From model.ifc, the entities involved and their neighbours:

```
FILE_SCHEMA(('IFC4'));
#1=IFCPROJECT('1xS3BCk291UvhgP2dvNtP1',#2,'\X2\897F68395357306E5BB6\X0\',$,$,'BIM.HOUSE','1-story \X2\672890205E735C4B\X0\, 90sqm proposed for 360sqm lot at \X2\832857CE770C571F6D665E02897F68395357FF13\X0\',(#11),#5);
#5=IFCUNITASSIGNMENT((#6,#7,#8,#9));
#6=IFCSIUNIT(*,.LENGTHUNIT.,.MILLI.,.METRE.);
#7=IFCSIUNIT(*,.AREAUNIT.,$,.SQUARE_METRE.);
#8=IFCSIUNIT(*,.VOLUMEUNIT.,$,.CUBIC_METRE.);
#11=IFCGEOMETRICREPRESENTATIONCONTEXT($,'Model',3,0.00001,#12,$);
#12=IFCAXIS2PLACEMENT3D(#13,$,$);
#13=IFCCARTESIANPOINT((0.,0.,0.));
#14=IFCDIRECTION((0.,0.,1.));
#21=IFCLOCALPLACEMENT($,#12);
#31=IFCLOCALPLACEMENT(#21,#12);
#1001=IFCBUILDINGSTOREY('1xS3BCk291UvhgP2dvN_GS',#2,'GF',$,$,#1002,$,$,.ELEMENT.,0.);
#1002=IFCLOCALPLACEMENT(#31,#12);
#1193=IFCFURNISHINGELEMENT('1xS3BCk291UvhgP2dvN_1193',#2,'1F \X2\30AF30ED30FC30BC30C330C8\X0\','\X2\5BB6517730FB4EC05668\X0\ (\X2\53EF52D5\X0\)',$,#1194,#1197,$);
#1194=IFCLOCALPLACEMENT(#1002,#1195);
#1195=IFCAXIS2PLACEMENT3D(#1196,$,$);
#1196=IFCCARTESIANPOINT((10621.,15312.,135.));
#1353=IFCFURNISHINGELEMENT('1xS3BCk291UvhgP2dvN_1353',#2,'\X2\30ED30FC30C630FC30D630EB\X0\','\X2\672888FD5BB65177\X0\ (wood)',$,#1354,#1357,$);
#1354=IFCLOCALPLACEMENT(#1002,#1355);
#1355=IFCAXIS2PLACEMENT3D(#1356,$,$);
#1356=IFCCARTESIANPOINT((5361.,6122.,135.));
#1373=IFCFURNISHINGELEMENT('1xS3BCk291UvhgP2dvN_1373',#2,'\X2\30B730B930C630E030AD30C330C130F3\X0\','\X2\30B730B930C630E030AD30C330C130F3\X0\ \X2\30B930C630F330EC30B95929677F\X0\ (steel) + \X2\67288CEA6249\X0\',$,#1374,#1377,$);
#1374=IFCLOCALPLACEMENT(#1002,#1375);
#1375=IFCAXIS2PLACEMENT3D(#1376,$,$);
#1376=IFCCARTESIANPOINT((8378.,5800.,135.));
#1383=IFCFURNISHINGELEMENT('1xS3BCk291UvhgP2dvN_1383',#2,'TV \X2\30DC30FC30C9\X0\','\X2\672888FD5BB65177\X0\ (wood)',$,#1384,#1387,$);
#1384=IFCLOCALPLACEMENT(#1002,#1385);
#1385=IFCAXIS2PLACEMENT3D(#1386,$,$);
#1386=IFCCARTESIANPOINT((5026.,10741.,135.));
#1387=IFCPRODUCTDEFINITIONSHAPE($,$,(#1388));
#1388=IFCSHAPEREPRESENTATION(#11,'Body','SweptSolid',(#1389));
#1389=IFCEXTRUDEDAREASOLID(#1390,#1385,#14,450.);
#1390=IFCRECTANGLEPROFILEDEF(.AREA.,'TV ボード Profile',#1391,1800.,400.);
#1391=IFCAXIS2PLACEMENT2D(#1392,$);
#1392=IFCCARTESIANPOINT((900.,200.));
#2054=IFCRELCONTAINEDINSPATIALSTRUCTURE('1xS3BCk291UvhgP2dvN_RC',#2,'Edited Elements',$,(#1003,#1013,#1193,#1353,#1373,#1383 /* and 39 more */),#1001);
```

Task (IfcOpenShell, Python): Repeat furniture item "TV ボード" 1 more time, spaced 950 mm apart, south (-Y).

```python
import numpy as np
import ifcopenshell
import ifcopenshell.api.geometry
import ifcopenshell.api.root
import ifcopenshell.util.element
import ifcopenshell.util.placement
import ifcopenshell.util.unit

model = ifcopenshell.open("model.ifc")
unit_scale = ifcopenshell.util.unit.calculate_unit_scale(model)


def reuse_history(source, copy):
    """copy_class also copies each property set's owner history, people and application; keep the originals."""
    for rel in copy.IsDefinedBy:
        if rel.is_a("IfcRelDefinesByProperties") and (history := rel.RelatingPropertyDefinition.OwnerHistory):
            rel.RelatingPropertyDefinition.OwnerHistory = source.OwnerHistory
            ifcopenshell.util.element.remove_deep2(model, history)


source = model.by_id(1383)
base = ifcopenshell.util.placement.get_local_placement(source.ObjectPlacement)
step = np.array([0.0, -1.0, 0.0]) * 0.95 / unit_scale

for i in range(1, 2):
    copy = ifcopenshell.api.root.copy_class(model, product=source)
    copy.Representation = ifcopenshell.util.element.copy_deep(
        model, source.Representation, exclude=["IfcGeometricRepresentationContext", "IfcRepresentationMap"]
    )
    reuse_history(source, copy)
    matrix = base.copy()
    matrix[:3, 3] += i * step
    print("added at", matrix[:3, 3].round(3) + 0.0)
    ifcopenshell.api.geometry.edit_object_placement(model, product=copy, matrix=matrix, is_si=False)

model.write("model_edited.ifc")
```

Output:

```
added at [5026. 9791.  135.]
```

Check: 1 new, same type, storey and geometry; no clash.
